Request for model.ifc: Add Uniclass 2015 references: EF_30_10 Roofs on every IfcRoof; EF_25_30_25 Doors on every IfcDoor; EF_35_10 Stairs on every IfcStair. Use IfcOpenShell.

First a look at what the model holds.

```python
import ifcopenshell

model = ifcopenshell.open("model.ifc")
print(model.schema)
print("classifications:", [c.Name for c in model.by_type("IfcClassification")])
for ifc_class in ("IfcDoor", "IfcRoof", "IfcStair", "IfcWall", "IfcWindow"):
    print(ifc_class, len(model.by_type(ifc_class)))
```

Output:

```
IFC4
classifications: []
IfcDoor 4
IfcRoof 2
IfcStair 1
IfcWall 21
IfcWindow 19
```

```python
import ifcopenshell
import ifcopenshell.api.classification

model = ifcopenshell.open("model.ifc")

system = ifcopenshell.api.classification.add_classification(model, classification="Uniclass 2015")

codes = {
    "IfcRoof": ("EF_30_10", "Roofs"),
    "IfcDoor": ("EF_25_30_25", "Doors"),
    "IfcStair": ("EF_35_10", "Stairs"),
}
for ifc_class, (code, name) in codes.items():
    products = model.by_type(ifc_class)
    ifcopenshell.api.classification.add_reference(
        model, products=products, classification=system, identification=code, name=name
    )
    print(code, len(products))

model.write("model-out.ifc")
```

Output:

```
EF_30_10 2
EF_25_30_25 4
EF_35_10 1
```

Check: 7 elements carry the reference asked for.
